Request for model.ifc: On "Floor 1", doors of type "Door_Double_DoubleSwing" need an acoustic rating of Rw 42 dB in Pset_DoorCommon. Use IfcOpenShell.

First a look at what the model holds.

```python
import ifcopenshell
import ifcopenshell.util.element

model = ifcopenshell.open("model.ifc")
print(model.schema)
storey = next(s for s in model.by_type("IfcBuildingStorey") if s.Name == "Floor 1")
doors = [e for e in ifcopenshell.util.element.get_decomposition(storey) if e.is_a("IfcDoor")]
seen = {}
for e in doors:
    element_type = ifcopenshell.util.element.get_type(e)
    key = (element_type.Name if element_type != e and element_type else None, ifcopenshell.util.element.get_pset(e, "Pset_DoorCommon", "AcousticRating"))
    seen[key] = seen.get(key, 0) + 1
for (name, value), count in sorted(seen.items(), key=str):
    print(count, "x", name, "|", value)
```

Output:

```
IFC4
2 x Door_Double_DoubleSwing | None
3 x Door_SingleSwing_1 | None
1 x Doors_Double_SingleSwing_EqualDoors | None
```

```python
import ifcopenshell
import ifcopenshell.api.pset
import ifcopenshell.util.element

model = ifcopenshell.open("model.ifc")

storey = next(s for s in model.by_type("IfcBuildingStorey") if s.Name == "Floor 1")
doors = [e for e in ifcopenshell.util.element.get_decomposition(storey) if e.is_a("IfcDoor")]

count = 0
for e in doors:
    element_type = ifcopenshell.util.element.get_type(e)
    if element_type in (None, e) or element_type.Name != "Door_Double_DoubleSwing":
        continue
    # add_pset returns the element's existing set when there is one.
    pset = ifcopenshell.api.pset.add_pset(model, product=e, name="Pset_DoorCommon")
    ifcopenshell.api.pset.edit_pset(model, pset=pset, properties={"AcousticRating": "Rw 42 dB"})
    count += 1

print(count, "doors updated")

model.write("model_updated.ifc")
```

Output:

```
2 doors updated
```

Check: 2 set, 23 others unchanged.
